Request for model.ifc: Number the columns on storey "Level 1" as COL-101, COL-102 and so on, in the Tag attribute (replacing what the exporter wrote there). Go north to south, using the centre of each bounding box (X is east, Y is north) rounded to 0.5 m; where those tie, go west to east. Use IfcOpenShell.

First a look at what the model holds.

```python
import ifcopenshell
import ifcopenshell.util.element
import ifcopenshell.util.placement

model = ifcopenshell.open("model.ifc")
print(model.schema)
storey = next(s for s in model.by_type("IfcBuildingStorey") if s.Name == "Level 1")
columns = [e for e in ifcopenshell.util.element.get_decomposition(storey) if e.is_a("IfcColumn")]
for e in sorted(columns, key=lambda e: e.id()):
    origin = ifcopenshell.util.placement.get_local_placement(e.ObjectPlacement)[:3, 3]
    print(e.id(), e.Tag, e.Name, origin.round(2) + 0.0, sep=" | ")
```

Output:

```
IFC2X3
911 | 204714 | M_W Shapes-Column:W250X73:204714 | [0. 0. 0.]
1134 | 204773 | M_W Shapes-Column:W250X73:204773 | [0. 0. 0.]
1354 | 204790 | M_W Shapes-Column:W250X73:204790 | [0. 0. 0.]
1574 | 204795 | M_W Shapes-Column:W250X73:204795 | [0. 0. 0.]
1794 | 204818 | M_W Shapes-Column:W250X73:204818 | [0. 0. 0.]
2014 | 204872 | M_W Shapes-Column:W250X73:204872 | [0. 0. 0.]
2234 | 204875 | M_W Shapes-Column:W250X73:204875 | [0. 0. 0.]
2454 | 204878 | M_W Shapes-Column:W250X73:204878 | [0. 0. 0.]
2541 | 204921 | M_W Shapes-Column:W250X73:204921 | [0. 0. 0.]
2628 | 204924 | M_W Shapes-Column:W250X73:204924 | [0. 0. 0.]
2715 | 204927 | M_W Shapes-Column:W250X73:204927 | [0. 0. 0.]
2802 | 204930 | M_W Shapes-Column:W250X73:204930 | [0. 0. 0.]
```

```python
import ifcopenshell
import ifcopenshell.geom
import ifcopenshell.util.element
import ifcopenshell.util.shape

model = ifcopenshell.open("model.ifc")
settings = ifcopenshell.geom.settings()
settings.set("use-world-coords", True)


def centre(element):
    shape = ifcopenshell.geom.create_shape(settings, element)
    return ifcopenshell.util.shape.get_bbox_centroid(shape.geometry)


storey = next(s for s in model.by_type("IfcBuildingStorey") if s.Name == "Level 1")
columns = [e for e in ifcopenshell.util.element.get_decomposition(storey) if e.is_a("IfcColumn")]

# Insertion points can sit at a corner or the storey origin, so sort by the geometry (in metres).
centres = {e: centre(e) for e in columns}
columns.sort(key=lambda e: (-round(centres[e][1] / 0.5), centres[e][0]))

for i, e in enumerate(columns, start=1):
    number = f"COL-1{i:02d}"
    e.Tag = number
    print(e.id(), number)

model.write("model-out.ifc")
```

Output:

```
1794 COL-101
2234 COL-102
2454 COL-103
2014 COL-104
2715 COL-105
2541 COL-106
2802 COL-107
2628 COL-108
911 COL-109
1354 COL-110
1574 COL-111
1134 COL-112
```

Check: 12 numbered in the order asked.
